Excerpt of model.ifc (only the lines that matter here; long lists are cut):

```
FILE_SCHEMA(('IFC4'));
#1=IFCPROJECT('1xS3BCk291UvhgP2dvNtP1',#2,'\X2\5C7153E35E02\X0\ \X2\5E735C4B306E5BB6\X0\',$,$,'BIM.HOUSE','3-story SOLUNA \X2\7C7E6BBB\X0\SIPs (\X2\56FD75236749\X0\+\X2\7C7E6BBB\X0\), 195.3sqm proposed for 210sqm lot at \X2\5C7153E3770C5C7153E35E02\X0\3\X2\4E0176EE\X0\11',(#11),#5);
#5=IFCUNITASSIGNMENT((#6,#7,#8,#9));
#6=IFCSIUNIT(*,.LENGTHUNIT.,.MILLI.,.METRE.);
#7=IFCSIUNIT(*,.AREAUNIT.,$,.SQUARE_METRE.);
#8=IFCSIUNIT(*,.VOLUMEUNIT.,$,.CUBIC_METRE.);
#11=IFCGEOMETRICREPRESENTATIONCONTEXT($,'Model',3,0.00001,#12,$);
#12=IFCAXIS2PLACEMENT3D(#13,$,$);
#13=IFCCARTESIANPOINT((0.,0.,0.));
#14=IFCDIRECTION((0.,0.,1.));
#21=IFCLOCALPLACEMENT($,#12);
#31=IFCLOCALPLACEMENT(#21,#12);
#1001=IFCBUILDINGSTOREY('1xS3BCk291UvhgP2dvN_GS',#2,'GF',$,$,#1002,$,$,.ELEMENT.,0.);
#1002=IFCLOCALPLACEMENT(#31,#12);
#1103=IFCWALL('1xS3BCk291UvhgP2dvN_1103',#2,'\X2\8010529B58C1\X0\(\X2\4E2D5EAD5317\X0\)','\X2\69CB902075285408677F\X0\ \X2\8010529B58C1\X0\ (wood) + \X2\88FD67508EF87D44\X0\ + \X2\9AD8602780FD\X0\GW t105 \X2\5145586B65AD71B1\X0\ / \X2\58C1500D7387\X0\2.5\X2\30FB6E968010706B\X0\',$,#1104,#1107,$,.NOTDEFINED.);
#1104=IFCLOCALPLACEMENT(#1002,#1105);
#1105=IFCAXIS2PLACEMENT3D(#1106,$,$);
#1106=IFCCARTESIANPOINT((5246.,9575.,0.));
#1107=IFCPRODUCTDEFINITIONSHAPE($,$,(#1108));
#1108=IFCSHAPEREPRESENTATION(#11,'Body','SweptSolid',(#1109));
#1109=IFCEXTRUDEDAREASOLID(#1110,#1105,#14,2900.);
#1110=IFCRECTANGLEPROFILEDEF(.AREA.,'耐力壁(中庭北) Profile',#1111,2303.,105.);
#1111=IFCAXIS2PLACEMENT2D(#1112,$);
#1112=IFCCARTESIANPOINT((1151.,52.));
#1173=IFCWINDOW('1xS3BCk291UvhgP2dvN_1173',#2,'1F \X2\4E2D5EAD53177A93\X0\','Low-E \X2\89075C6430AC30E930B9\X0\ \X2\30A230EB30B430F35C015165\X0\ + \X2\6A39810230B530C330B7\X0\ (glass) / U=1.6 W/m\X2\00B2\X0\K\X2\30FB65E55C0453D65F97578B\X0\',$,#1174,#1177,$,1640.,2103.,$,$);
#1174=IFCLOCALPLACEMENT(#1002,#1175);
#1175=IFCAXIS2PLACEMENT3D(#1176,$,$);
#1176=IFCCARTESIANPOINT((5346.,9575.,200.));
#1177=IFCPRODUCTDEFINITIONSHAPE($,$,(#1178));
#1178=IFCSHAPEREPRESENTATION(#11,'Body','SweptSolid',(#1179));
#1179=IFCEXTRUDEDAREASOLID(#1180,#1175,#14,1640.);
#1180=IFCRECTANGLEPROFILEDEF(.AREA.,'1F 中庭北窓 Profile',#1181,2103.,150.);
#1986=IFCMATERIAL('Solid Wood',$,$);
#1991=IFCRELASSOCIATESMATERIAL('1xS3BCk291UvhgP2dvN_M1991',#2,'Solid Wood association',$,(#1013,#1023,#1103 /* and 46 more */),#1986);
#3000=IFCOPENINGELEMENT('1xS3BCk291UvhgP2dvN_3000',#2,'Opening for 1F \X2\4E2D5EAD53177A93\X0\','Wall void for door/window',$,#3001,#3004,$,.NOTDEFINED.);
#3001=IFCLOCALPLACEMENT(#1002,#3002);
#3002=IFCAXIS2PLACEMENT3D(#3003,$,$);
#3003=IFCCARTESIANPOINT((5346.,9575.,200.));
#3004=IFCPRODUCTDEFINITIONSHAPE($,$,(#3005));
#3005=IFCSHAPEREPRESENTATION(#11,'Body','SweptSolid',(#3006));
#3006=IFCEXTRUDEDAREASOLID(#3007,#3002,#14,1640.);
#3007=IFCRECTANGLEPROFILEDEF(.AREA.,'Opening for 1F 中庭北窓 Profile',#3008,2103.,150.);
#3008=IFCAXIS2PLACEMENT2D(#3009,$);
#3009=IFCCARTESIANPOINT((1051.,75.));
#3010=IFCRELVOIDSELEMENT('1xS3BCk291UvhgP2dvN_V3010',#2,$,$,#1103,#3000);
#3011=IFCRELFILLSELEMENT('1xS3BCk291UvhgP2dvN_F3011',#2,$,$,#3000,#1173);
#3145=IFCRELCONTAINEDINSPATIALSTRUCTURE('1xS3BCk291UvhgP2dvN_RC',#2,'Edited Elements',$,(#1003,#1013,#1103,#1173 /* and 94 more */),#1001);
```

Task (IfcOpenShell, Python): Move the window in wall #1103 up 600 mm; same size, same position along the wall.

```python
import numpy as np
import ifcopenshell
import ifcopenshell.api.geometry
import ifcopenshell.util.placement
import ifcopenshell.util.unit

model = ifcopenshell.open("model.ifc")
unit_scale = ifcopenshell.util.unit.calculate_unit_scale(model)

window = model.by_id(1173)
opening = window.FillsVoids[0].RelatingOpeningElement
dz = 0.6 / unit_scale

shift = np.array([0.0, 0.0, dz])
# The window is not placed relative to its opening, so move both.
for product in (opening, window):
    matrix = ifcopenshell.util.placement.get_local_placement(product.ObjectPlacement)
    matrix[:3, 3] += shift
    ifcopenshell.api.geometry.edit_object_placement(model, product=product, matrix=matrix, is_si=False)

print(f"moved by {dz * unit_scale:+.3f} m")

model.write("model_edited.ifc")
```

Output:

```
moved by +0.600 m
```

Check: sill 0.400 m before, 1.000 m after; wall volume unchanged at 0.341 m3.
